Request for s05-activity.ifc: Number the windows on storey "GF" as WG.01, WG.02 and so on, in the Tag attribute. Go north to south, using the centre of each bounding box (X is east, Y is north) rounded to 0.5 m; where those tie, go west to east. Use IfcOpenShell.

First a look at what the model holds.

```python
import ifcopenshell
import ifcopenshell.util.element
import ifcopenshell.util.placement

model = ifcopenshell.open("s05-activity.ifc")
print(model.schema)
storey = next(s for s in model.by_type("IfcBuildingStorey") if s.Name == "GF")
windows = [e for e in ifcopenshell.util.element.get_decomposition(storey) if e.is_a("IfcWindow")]
for e in sorted(windows, key=lambda e: e.id()):
    origin = ifcopenshell.util.placement.get_local_placement(e.ObjectPlacement)[:3, 3]
    print(e.id(), e.Tag, e.Name, origin.round(2) + 0.0, sep=" | ")
```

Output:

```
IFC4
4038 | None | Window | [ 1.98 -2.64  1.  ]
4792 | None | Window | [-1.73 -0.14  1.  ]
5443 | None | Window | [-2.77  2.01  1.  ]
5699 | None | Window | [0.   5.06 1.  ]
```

```python
import ifcopenshell
import ifcopenshell.geom
import ifcopenshell.util.element
import ifcopenshell.util.shape

model = ifcopenshell.open("s05-activity.ifc")
settings = ifcopenshell.geom.settings()
settings.set("use-world-coords", True)


def centre(element):
    shape = ifcopenshell.geom.create_shape(settings, element)
    return ifcopenshell.util.shape.get_bbox_centroid(shape.geometry)


storey = next(s for s in model.by_type("IfcBuildingStorey") if s.Name == "GF")
windows = [e for e in ifcopenshell.util.element.get_decomposition(storey) if e.is_a("IfcWindow")]

# Insertion points can sit at a corner or the storey origin, so sort by the geometry (in metres).
centres = {e: centre(e) for e in windows}
windows.sort(key=lambda e: (-round(centres[e][1] / 0.5), centres[e][0]))

for i, e in enumerate(windows, start=1):
    number = f"WG.{i:02d}"
    e.Tag = number
    print(e.id(), number)

model.write("s05-activity_edited.ifc")
```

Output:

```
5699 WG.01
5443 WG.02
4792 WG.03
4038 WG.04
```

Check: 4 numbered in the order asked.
